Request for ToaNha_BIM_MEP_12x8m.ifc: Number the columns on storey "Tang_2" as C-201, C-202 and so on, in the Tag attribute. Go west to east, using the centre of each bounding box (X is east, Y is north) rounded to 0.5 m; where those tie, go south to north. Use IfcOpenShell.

First a look at what the model holds.

```python
import ifcopenshell
import ifcopenshell.util.element
import ifcopenshell.util.placement

model = ifcopenshell.open("ToaNha_BIM_MEP_12x8m.ifc")
print(model.schema)
storey = next(s for s in model.by_type("IfcBuildingStorey") if s.Name == "Tang_2")
columns = [e for e in ifcopenshell.util.element.get_decomposition(storey) if e.is_a("IfcColumn")]
for e in sorted(columns, key=lambda e: e.id()):
    origin = ifcopenshell.util.placement.get_local_placement(e.ObjectPlacement)[:3, 3]
    print(e.id(), e.Tag, e.Name, origin.round(2) + 0.0, sep=" | ")
```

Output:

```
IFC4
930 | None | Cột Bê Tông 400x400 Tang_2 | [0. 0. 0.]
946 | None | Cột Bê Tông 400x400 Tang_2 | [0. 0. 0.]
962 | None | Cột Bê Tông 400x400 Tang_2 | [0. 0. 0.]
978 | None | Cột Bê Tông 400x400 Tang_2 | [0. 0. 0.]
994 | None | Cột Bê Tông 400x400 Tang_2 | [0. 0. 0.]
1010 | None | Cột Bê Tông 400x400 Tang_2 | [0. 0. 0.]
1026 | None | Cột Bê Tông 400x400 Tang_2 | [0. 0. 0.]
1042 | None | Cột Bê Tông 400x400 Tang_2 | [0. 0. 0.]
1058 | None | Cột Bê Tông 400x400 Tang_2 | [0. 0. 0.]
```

```python
import ifcopenshell
import ifcopenshell.geom
import ifcopenshell.util.element
import ifcopenshell.util.shape

model = ifcopenshell.open("ToaNha_BIM_MEP_12x8m.ifc")
settings = ifcopenshell.geom.settings()
settings.set("use-world-coords", True)


def centre(element):
    shape = ifcopenshell.geom.create_shape(settings, element)
    return ifcopenshell.util.shape.get_bbox_centroid(shape.geometry)


storey = next(s for s in model.by_type("IfcBuildingStorey") if s.Name == "Tang_2")
columns = [e for e in ifcopenshell.util.element.get_decomposition(storey) if e.is_a("IfcColumn")]

# Insertion points can sit at a corner or the storey origin, so sort by the geometry (in metres).
centres = {e: centre(e) for e in columns}
columns.sort(key=lambda e: (round(centres[e][0] / 0.5), centres[e][1]))

for i, e in enumerate(columns, start=1):
    number = f"C-2{i:02d}"
    e.Tag = number
    print(e.id(), number)

model.write("ToaNha_BIM_MEP_12x8m-out.ifc")
```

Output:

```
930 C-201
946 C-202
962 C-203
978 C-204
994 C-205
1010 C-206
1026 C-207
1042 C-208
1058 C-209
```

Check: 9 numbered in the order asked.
